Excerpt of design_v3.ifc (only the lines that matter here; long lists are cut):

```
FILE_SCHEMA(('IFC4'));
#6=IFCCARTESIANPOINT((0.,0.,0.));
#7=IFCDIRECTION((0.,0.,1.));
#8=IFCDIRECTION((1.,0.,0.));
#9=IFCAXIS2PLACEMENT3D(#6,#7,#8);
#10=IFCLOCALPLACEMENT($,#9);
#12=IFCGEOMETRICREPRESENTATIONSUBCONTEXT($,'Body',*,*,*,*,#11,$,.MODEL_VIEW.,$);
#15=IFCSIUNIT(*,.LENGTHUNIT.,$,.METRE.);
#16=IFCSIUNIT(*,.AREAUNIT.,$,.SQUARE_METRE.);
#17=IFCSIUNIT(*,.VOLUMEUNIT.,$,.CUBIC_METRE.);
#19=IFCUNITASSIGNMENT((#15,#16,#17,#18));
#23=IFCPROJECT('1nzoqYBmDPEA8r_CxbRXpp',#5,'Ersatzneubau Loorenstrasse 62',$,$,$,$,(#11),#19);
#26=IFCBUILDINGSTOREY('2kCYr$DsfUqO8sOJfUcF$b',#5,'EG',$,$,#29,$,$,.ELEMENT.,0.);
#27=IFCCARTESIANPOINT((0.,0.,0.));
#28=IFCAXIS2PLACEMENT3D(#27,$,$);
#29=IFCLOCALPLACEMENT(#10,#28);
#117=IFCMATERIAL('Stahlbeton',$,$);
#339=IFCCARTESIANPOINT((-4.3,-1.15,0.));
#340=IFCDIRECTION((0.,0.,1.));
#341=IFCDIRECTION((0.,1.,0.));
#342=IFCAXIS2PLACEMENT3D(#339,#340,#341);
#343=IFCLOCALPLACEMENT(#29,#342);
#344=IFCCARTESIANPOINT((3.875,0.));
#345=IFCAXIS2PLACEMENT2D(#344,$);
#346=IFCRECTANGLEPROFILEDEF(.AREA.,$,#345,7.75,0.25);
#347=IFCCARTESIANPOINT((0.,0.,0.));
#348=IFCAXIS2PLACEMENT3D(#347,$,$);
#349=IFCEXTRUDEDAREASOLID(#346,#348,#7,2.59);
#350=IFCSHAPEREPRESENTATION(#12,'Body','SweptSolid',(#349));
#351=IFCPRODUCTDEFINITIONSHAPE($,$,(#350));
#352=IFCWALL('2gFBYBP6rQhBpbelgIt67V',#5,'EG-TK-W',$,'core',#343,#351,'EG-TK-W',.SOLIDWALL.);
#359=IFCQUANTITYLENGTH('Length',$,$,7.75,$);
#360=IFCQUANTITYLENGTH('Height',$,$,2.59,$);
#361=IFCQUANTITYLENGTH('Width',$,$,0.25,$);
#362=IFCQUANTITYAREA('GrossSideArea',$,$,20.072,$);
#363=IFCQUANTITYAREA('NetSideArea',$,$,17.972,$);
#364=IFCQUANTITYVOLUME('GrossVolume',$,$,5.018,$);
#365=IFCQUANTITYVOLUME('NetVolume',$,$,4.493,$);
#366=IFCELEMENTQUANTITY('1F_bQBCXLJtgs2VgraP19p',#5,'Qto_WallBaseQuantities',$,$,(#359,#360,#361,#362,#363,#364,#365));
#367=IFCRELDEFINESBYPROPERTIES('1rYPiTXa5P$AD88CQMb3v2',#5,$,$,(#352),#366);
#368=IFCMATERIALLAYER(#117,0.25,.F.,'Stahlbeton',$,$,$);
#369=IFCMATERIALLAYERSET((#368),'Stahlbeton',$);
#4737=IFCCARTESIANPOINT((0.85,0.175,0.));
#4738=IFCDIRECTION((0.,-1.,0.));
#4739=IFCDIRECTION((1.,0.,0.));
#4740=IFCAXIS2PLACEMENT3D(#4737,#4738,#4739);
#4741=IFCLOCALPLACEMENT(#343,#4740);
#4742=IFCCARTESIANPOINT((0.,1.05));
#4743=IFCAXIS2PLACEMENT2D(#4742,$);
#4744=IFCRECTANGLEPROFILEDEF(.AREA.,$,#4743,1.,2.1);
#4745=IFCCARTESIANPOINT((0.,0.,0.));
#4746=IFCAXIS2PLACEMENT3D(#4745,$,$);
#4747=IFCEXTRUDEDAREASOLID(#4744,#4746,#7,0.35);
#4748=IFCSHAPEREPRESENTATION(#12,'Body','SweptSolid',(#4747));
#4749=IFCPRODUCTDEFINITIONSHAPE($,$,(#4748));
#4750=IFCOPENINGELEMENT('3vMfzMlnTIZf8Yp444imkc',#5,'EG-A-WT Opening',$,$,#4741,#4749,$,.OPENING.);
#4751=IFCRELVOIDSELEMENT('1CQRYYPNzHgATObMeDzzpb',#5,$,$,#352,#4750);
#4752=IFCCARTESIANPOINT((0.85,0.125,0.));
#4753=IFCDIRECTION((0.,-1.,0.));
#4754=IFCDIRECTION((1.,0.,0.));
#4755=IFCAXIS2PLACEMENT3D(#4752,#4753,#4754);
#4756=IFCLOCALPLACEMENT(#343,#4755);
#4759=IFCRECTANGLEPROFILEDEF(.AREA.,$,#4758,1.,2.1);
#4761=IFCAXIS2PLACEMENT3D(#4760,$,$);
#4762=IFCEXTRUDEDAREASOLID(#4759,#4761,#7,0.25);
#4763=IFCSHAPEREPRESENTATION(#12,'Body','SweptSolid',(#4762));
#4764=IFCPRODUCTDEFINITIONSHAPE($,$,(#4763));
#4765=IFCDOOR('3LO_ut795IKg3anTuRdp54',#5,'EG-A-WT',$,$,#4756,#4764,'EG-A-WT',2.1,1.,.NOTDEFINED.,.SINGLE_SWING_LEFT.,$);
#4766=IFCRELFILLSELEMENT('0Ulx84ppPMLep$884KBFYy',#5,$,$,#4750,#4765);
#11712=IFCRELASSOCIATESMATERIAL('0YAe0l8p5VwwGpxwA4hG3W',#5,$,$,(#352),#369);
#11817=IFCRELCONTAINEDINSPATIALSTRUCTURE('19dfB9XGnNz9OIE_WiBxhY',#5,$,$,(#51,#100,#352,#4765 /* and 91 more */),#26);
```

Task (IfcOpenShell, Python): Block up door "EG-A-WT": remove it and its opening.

```python
import ifcopenshell
import ifcopenshell.api.feature
import ifcopenshell.api.pset
import ifcopenshell.api.root
import ifcopenshell.geom
import ifcopenshell.util.element
import ifcopenshell.util.shape
import ifcopenshell.util.unit

model = ifcopenshell.open("design_v3.ifc")
area_scale = ifcopenshell.util.unit.calculate_unit_scale(model, "AREAUNIT")
volume_scale = ifcopenshell.util.unit.calculate_unit_scale(model, "VOLUMEUNIT")
settings = ifcopenshell.geom.settings()


def volume(element):
    """Net volume in cubic metres, openings subtracted."""
    shape = ifcopenshell.geom.create_shape(settings, element)
    return ifcopenshell.util.shape.get_volume(shape.geometry)


door = model.by_guid("3LO_ut795IKg3anTuRdp54")
opening = door.FillsVoids[0].RelatingOpeningElement
wall = opening.VoidsElements[0].RelatingBuildingElement
before = volume(wall)

ifcopenshell.api.root.remove_product(model, product=door)
ifcopenshell.api.feature.remove_feature(model, feature=opening)

after = volume(wall)
thickness = 0.25  # wall thickness in metres

# Update the wall's stored quantities.
qto = model.by_id(ifcopenshell.util.element.get_pset(wall, "Qto_WallBaseQuantities", should_inherit=False)["id"])
ifcopenshell.api.pset.edit_qto(model, qto=qto, properties={
    "NetSideArea": after / thickness / area_scale,
    "NetVolume": after / volume_scale,
})

print(f"wall volume {before:.3f} -> {after:.3f} m3")

model.write("design_v3_v2.ifc")
```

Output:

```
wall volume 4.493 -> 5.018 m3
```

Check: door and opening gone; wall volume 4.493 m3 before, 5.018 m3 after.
